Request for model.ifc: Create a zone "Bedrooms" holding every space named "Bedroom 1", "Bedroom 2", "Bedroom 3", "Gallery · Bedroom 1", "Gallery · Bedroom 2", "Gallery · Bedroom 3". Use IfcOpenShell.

First a look at what the model holds.

```python
import ifcopenshell

model = ifcopenshell.open("model.ifc")
print(model.schema)
seen = {}
for space in model.by_type("IfcSpace"):
    seen[space.Name] = seen.get(space.Name, 0) + 1
for name, count in sorted(seen.items(), key=str):
    print(count, "x", name)
print("zones:", [z.Name for z in model.by_type("IfcZone")][:20])
```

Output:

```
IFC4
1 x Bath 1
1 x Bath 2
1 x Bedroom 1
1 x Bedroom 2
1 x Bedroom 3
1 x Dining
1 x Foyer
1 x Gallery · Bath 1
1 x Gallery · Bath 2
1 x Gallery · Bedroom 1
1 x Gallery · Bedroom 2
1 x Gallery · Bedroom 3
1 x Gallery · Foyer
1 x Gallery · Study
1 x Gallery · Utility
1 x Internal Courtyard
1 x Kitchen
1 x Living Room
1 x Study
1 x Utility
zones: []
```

```python
import ifcopenshell
import ifcopenshell.api.group
import ifcopenshell.api.root

model = ifcopenshell.open("model.ifc")

names = {"Bedroom 1", "Bedroom 2", "Bedroom 3", "Gallery · Bedroom 1", "Gallery · Bedroom 2", "Gallery · Bedroom 3"}
spaces = [s for s in model.by_type("IfcSpace") if s.Name in names]

zone = ifcopenshell.api.root.create_entity(model, ifc_class="IfcZone", name="Bedrooms")
ifcopenshell.api.group.assign_group(model, products=spaces, group=zone)
print(len(spaces), "spaces in", zone.Name)

model.write("model_v2.ifc")
```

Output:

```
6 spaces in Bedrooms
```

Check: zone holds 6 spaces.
